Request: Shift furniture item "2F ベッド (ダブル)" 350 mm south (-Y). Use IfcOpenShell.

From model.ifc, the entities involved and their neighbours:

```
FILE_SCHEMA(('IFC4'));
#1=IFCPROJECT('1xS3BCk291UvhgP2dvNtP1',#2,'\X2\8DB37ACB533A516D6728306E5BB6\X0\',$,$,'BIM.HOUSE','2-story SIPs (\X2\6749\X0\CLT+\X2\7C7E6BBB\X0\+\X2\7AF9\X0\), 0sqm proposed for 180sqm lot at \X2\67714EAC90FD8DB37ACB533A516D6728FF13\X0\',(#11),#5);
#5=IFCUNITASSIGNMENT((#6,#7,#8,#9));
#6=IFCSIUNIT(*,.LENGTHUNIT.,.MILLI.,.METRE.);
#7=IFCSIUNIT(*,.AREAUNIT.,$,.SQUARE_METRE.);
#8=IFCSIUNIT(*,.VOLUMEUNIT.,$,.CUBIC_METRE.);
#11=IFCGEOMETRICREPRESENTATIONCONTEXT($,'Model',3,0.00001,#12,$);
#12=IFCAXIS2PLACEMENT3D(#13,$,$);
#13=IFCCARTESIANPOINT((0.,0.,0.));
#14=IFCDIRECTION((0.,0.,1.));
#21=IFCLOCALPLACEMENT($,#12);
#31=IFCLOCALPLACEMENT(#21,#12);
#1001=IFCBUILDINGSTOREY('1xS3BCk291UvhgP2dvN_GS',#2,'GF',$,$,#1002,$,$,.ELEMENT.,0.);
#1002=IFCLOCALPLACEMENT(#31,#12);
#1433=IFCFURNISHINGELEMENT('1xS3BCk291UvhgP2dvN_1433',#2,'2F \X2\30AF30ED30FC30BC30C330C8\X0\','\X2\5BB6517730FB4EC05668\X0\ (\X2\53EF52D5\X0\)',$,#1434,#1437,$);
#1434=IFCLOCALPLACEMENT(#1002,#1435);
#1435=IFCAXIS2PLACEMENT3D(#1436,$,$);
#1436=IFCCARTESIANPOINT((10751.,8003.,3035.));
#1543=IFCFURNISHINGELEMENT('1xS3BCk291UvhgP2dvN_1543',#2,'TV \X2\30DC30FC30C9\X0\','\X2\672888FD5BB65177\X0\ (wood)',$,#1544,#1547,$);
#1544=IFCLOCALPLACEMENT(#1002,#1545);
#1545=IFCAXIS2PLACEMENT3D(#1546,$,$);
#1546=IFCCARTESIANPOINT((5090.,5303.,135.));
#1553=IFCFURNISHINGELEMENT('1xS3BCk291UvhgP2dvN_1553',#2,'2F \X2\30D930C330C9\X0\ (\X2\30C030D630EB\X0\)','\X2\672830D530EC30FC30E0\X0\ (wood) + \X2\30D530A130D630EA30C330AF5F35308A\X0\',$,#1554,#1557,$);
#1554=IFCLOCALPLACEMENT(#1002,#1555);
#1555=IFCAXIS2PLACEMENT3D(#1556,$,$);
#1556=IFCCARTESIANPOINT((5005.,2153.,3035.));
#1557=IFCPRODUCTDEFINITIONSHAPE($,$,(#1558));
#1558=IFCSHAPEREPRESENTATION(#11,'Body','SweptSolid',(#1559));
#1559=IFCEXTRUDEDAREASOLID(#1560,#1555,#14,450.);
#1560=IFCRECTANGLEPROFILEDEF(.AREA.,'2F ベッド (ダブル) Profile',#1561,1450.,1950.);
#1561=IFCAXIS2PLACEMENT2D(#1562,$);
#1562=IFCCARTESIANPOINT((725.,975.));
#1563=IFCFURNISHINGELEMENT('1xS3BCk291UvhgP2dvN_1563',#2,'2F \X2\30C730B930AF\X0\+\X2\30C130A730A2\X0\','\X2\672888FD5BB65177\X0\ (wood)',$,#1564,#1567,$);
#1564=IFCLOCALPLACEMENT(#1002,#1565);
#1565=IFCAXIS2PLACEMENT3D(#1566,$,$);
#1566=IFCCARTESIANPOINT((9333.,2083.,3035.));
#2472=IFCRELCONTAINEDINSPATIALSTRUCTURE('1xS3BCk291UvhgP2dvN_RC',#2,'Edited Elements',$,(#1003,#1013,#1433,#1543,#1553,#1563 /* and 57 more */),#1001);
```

```python
import ifcopenshell
import ifcopenshell.api.geometry
import ifcopenshell.util.placement

model = ifcopenshell.open("model.ifc")

item = model.by_guid("1xS3BCk291UvhgP2dvN_1553")
matrix = ifcopenshell.util.placement.get_local_placement(item.ObjectPlacement)
matrix[1, 3] -= 350.0
ifcopenshell.api.geometry.edit_object_placement(model, product=item, matrix=matrix, is_si=False)

print(ifcopenshell.util.placement.get_local_placement(item.ObjectPlacement).round(3) + 0.0)

model.write("model_updated.ifc")
```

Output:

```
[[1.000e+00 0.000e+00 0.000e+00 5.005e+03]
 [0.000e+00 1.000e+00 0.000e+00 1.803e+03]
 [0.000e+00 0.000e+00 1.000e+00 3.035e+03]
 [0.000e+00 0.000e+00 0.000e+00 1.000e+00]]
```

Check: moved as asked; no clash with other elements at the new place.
